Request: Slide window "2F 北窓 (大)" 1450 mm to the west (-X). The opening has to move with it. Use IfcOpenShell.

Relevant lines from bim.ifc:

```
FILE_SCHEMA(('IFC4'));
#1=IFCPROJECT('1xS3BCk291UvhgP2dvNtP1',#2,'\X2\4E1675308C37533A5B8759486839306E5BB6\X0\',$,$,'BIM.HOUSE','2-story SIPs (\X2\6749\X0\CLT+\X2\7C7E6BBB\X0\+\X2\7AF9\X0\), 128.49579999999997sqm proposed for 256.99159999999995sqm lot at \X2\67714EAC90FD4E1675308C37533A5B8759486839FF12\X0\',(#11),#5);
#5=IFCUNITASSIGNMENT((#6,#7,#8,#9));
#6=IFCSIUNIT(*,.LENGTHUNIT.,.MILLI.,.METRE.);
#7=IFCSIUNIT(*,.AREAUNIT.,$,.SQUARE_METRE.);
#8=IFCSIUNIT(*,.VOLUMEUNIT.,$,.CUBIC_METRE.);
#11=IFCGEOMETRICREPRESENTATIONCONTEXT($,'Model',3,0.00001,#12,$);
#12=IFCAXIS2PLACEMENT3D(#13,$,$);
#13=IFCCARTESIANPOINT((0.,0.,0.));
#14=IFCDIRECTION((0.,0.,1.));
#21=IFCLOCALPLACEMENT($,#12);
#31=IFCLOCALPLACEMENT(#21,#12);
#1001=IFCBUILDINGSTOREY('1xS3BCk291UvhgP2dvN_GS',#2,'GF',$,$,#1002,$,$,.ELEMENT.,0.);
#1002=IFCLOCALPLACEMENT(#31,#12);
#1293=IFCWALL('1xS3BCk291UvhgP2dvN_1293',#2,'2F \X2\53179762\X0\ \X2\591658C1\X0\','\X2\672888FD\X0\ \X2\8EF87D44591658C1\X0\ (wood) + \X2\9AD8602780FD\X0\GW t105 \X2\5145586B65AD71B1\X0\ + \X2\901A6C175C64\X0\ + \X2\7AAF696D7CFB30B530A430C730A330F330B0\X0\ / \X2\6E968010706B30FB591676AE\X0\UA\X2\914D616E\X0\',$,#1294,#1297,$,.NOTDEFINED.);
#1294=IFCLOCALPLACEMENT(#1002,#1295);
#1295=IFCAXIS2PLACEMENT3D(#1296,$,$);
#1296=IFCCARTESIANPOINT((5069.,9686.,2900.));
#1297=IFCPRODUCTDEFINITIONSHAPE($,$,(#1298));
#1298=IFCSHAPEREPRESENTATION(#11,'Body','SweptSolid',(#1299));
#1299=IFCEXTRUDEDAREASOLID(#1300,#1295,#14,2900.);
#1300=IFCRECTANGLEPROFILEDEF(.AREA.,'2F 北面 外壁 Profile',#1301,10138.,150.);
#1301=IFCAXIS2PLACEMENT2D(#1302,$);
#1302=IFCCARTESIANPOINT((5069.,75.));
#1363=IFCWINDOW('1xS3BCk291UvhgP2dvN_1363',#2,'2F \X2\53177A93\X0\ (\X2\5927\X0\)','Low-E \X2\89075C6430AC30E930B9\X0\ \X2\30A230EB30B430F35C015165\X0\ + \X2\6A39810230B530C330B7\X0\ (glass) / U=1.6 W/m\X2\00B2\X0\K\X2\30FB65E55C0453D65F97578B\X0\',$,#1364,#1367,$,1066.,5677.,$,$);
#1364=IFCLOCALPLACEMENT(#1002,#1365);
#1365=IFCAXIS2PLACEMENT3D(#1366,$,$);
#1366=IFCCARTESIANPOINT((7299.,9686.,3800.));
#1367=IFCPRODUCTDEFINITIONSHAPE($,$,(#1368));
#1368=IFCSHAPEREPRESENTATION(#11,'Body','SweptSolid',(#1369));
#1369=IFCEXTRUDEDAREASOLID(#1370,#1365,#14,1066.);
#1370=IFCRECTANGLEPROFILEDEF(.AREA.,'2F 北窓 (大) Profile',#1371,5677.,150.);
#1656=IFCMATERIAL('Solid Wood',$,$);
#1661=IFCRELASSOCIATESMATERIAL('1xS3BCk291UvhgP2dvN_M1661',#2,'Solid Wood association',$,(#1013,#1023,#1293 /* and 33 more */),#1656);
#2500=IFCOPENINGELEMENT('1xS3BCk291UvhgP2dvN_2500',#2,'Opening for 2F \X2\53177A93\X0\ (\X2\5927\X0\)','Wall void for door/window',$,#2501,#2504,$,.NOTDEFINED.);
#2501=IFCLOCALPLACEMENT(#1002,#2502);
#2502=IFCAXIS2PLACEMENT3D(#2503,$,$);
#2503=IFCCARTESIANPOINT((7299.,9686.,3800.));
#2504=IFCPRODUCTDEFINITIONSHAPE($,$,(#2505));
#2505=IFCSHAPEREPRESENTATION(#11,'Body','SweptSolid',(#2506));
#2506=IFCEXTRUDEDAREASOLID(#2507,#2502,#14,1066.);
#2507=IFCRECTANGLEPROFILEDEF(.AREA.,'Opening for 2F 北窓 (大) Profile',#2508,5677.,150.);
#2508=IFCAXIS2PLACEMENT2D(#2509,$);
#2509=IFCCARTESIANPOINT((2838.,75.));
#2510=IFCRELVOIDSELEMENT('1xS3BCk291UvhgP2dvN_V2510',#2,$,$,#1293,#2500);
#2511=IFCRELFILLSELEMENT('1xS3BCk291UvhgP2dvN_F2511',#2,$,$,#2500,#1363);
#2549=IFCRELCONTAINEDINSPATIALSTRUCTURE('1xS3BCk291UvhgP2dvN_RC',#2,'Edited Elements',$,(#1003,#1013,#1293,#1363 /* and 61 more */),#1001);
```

```python
import ifcopenshell
import ifcopenshell.api.geometry
import ifcopenshell.util.placement
import ifcopenshell.util.unit

model = ifcopenshell.open("bim.ifc")
unit_scale = ifcopenshell.util.unit.calculate_unit_scale(model)

window = model.by_id(1363)
opening = window.FillsVoids[0].RelatingOpeningElement
wall = opening.VoidsElements[0].RelatingBuildingElement

wall_matrix = ifcopenshell.util.placement.get_local_placement(wall.ObjectPlacement)
shift = wall_matrix[:3, 0] * -1.45 / unit_scale
before = ifcopenshell.util.placement.get_local_placement(window.ObjectPlacement)[:3, 3].copy()

# The window is not placed relative to its opening, so move both.
for product in (opening, window):
    matrix = ifcopenshell.util.placement.get_local_placement(product.ObjectPlacement)
    matrix[:3, 3] += shift
    ifcopenshell.api.geometry.edit_object_placement(model, product=product, matrix=matrix, is_si=False)

after = ifcopenshell.util.placement.get_local_placement(window.ObjectPlacement)[:3, 3]
print("window moved by", (after - before).round(3) + 0.0)

model.write("bim-out.ifc")
```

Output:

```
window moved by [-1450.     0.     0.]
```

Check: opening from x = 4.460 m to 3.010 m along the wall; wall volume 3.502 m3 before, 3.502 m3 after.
